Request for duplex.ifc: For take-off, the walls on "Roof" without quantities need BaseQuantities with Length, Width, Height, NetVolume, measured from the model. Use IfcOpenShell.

First a look at what the model holds.

```python
import ifcopenshell
import ifcopenshell.util.element
import ifcopenshell.util.unit

model = ifcopenshell.open("duplex.ifc")
print(model.schema)
for unit_type in ("LENGTHUNIT", "AREAUNIT", "VOLUMEUNIT"):
    print(unit_type, ifcopenshell.util.unit.calculate_unit_scale(model, unit_type))
storey = next(s for s in model.by_type("IfcBuildingStorey") if s.Name == "Roof")
walls = [e for e in ifcopenshell.util.element.get_decomposition(storey) if e.is_a("IfcWall")]
for e in sorted(walls, key=lambda e: e.id()):
    print(e.id(), e.is_a(), e.Name, list(ifcopenshell.util.element.get_psets(e, qtos_only=True)), sep=" | ")
```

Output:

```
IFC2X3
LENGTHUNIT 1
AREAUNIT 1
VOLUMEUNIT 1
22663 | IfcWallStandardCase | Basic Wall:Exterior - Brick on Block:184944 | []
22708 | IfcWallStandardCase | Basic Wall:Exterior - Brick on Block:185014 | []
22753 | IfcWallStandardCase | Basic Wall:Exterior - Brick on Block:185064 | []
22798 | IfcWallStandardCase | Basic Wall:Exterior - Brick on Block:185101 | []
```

```python
import ifcopenshell
import ifcopenshell.api.pset
import ifcopenshell.geom
import ifcopenshell.util.element
import ifcopenshell.util.shape
import ifcopenshell.util.unit

model = ifcopenshell.open("duplex.ifc")
unit_scale = ifcopenshell.util.unit.calculate_unit_scale(model)
volume_scale = ifcopenshell.util.unit.calculate_unit_scale(model, "VOLUMEUNIT")
settings = ifcopenshell.geom.settings()

storey = next(s for s in model.by_type("IfcBuildingStorey") if s.Name == "Roof")
walls = [e for e in ifcopenshell.util.element.get_decomposition(storey) if e.is_a("IfcWall")]

for e in sorted(walls, key=lambda e: e.id()):
    if ifcopenshell.util.element.get_psets(e, qtos_only=True, should_inherit=False):
        continue
    # Geometry comes back in metres, in the element's own axes.
    shape = ifcopenshell.geom.create_shape(settings, e)
    values = {
        "Length": ifcopenshell.util.shape.get_x(shape.geometry) / unit_scale,
        "Width": ifcopenshell.util.shape.get_y(shape.geometry) / unit_scale,
        "Height": ifcopenshell.util.shape.get_z(shape.geometry) / unit_scale,
        "NetVolume": ifcopenshell.util.shape.get_volume(shape.geometry) / volume_scale,
    }
    qto = ifcopenshell.api.pset.add_qto(model, product=e, name="BaseQuantities")
    ifcopenshell.api.pset.edit_qto(model, qto=qto, properties=values)
    print(e.id(), {k: round(v, 3) for k, v in values.items()})

model.write("duplex-out.ifc")
```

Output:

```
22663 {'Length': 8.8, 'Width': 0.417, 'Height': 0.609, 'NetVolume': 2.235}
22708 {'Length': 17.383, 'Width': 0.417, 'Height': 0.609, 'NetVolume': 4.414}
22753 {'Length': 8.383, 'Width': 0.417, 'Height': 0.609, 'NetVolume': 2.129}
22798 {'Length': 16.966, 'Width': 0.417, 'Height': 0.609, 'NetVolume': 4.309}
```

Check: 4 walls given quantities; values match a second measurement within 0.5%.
